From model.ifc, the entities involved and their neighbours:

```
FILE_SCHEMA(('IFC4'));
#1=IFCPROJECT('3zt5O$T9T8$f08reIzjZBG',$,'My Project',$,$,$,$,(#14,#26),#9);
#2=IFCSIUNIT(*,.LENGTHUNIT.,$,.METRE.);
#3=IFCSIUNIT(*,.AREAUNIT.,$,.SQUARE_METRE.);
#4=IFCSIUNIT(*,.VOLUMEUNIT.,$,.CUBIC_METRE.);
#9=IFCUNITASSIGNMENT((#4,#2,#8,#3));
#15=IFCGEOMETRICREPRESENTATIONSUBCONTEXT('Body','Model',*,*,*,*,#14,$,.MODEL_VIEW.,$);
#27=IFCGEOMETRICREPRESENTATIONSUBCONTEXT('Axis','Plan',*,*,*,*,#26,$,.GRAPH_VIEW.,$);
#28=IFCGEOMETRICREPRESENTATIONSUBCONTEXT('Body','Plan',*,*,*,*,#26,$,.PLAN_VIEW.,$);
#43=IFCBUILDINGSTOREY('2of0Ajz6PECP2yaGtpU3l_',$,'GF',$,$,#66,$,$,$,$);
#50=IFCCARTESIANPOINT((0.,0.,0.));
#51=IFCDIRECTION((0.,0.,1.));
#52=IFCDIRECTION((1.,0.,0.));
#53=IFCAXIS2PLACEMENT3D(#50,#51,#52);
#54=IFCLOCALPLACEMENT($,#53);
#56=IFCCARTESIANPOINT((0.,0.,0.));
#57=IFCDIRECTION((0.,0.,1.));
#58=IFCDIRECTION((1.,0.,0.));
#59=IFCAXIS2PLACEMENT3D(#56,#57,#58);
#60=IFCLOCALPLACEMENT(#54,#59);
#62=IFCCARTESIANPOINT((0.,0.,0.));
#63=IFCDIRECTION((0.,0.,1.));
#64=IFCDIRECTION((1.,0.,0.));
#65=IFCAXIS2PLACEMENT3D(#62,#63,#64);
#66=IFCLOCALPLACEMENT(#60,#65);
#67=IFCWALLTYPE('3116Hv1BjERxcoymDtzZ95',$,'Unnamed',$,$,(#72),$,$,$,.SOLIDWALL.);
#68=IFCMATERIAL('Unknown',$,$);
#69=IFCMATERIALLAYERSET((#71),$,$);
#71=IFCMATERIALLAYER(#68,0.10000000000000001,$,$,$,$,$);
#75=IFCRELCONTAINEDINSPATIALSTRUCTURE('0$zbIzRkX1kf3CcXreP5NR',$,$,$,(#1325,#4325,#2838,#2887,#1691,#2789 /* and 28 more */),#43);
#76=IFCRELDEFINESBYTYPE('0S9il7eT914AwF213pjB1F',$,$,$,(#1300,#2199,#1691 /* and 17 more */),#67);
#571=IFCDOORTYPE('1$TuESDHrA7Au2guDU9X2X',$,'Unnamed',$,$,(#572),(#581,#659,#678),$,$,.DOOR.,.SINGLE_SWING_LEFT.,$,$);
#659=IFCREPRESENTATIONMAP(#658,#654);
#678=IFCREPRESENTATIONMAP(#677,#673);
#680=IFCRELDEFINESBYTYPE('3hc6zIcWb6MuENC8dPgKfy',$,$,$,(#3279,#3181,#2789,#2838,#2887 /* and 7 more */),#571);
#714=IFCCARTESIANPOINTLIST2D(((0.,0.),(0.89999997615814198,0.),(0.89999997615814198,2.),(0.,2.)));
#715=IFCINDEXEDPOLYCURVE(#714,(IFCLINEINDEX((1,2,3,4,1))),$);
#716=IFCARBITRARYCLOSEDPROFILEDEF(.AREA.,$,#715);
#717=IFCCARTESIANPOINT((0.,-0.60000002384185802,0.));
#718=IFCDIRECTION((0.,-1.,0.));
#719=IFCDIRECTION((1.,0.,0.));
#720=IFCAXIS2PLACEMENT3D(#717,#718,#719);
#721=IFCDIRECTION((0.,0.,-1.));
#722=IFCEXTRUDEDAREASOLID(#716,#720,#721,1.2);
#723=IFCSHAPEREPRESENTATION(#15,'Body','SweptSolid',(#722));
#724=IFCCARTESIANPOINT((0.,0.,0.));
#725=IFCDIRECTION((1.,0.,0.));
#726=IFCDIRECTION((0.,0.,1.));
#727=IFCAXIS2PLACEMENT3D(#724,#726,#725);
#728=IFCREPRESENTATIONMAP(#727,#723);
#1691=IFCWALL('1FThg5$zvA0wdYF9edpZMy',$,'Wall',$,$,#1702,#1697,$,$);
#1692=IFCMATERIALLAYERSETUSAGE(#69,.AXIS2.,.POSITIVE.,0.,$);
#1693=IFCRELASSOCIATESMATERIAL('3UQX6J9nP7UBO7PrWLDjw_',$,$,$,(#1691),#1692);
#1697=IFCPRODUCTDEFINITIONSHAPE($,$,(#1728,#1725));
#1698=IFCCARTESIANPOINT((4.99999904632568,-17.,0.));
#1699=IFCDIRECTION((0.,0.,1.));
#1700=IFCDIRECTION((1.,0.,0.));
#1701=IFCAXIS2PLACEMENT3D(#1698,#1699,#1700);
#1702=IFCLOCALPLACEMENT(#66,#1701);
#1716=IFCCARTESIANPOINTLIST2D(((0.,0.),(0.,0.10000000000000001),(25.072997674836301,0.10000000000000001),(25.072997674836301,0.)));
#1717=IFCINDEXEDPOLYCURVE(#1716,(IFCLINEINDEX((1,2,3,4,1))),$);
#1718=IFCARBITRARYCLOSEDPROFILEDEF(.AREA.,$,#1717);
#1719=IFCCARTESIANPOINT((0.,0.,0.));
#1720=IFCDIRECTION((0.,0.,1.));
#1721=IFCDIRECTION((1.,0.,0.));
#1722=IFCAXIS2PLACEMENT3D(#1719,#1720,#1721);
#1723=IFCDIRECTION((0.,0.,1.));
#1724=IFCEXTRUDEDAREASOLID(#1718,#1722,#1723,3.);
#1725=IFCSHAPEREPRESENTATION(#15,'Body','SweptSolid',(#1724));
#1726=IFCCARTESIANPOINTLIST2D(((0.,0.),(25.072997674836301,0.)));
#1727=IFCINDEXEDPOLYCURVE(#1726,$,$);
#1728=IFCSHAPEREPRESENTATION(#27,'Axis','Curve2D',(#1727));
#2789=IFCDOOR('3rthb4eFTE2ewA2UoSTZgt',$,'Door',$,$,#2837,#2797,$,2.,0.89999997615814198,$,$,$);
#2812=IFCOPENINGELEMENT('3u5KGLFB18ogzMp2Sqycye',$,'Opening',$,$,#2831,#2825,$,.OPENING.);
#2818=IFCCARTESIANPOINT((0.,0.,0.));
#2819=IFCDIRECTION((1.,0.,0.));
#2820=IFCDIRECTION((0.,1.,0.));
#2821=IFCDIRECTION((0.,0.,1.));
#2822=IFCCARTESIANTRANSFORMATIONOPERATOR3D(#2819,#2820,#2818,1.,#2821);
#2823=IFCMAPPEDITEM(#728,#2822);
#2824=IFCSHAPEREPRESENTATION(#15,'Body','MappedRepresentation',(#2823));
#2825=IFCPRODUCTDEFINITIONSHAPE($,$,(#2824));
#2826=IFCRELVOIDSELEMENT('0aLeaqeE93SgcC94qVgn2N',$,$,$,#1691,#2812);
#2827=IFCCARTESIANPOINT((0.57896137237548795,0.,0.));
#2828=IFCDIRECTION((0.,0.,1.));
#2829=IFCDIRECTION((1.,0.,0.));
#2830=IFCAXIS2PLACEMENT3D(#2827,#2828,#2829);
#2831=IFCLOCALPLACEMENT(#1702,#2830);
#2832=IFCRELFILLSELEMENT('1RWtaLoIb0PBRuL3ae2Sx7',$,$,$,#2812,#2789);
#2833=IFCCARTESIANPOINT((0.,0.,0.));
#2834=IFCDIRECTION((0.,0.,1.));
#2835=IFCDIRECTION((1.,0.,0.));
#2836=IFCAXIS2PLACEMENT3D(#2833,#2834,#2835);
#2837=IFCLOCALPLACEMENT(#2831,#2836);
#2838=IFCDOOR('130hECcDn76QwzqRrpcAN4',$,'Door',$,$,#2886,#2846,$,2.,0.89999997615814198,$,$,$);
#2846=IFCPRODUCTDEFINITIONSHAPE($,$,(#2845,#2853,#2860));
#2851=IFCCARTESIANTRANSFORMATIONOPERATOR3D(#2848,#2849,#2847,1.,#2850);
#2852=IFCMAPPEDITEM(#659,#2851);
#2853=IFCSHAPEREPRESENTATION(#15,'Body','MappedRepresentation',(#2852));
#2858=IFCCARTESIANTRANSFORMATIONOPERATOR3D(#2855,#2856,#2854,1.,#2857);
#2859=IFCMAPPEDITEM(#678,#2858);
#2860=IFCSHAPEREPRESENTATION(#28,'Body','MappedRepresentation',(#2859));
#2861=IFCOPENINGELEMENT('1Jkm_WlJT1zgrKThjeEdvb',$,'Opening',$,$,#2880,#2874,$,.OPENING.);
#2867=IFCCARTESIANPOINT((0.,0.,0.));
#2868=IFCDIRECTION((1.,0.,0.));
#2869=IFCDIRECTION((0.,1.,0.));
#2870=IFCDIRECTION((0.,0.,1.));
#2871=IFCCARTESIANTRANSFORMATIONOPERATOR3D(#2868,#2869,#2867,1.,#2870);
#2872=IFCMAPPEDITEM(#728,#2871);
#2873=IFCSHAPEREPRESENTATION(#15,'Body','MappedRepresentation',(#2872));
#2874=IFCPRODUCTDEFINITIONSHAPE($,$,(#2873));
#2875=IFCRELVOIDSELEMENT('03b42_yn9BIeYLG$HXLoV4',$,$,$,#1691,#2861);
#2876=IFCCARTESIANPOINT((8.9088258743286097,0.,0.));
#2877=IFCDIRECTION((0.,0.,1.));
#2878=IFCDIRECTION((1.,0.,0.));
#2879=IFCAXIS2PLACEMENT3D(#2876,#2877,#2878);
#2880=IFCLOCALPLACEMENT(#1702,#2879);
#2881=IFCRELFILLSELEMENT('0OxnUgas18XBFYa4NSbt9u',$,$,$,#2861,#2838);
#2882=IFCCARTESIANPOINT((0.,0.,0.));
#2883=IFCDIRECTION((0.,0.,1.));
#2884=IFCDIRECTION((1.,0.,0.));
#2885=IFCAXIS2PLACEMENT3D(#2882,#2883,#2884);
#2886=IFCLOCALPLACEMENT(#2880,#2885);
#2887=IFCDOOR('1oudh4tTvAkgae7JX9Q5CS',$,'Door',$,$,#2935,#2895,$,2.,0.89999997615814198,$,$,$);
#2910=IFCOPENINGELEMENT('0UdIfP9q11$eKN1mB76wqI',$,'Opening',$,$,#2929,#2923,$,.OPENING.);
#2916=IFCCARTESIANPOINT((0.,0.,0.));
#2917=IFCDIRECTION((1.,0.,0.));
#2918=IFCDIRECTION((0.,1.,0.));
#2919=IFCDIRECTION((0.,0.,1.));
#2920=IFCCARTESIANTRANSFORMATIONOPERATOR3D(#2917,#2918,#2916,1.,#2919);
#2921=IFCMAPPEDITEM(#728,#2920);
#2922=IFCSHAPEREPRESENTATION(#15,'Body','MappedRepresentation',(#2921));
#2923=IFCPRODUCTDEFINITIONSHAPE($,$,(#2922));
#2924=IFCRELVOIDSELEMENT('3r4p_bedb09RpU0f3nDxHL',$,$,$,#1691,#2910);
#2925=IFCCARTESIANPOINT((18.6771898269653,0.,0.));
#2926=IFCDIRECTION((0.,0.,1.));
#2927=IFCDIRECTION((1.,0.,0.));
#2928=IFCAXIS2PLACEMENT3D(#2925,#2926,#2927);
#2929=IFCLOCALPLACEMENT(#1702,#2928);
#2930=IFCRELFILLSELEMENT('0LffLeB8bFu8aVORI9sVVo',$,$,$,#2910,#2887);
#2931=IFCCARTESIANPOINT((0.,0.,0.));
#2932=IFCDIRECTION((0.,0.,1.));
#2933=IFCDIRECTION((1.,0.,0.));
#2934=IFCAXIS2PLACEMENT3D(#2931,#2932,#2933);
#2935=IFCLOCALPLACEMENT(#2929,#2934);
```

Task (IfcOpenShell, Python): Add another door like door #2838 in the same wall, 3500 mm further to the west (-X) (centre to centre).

```python
import ifcopenshell
import ifcopenshell.api.feature
import ifcopenshell.api.geometry
import ifcopenshell.api.root
import ifcopenshell.geom
import ifcopenshell.util.element
import ifcopenshell.util.placement
import ifcopenshell.util.shape

model = ifcopenshell.open("model.ifc")
settings = ifcopenshell.geom.settings()


def volume(element):
    """Net volume in cubic metres, openings subtracted."""
    shape = ifcopenshell.geom.create_shape(settings, element)
    return ifcopenshell.util.shape.get_volume(shape.geometry)


door = model.by_guid("130hECcDn76QwzqRrpcAN4")
opening = door.FillsVoids[0].RelatingOpeningElement
wall = opening.VoidsElements[0].RelatingBuildingElement
before = volume(wall)
shift = ifcopenshell.util.placement.get_local_placement(wall.ObjectPlacement)[:3, 0] * -3.5

# copy_class copies the void relationship, type, container and properties, but no geometry.
new_opening = ifcopenshell.api.root.copy_class(model, product=opening)
new_opening.Representation = ifcopenshell.util.element.copy_deep(
    model, opening.Representation, exclude=["IfcGeometricRepresentationContext", "IfcRepresentationMap"]
)
new_door = ifcopenshell.api.root.copy_class(model, product=door)
new_door.Representation = ifcopenshell.util.element.copy_deep(
    model, door.Representation, exclude=["IfcGeometricRepresentationContext", "IfcRepresentationMap"]
)
ifcopenshell.api.feature.add_filling(model, opening=new_opening, element=new_door)

for old, new in ((opening, new_opening), (door, new_door)):
    matrix = ifcopenshell.util.placement.get_local_placement(old.ObjectPlacement)
    matrix[:3, 3] += shift
    ifcopenshell.api.geometry.edit_object_placement(model, product=new, matrix=matrix, is_si=False)

after = volume(wall)

print(f"wall volume {before:.3f} -> {after:.3f} m3")

model.write("model_edited.ifc")
```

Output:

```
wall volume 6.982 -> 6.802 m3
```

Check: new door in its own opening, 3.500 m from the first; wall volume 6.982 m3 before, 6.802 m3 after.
